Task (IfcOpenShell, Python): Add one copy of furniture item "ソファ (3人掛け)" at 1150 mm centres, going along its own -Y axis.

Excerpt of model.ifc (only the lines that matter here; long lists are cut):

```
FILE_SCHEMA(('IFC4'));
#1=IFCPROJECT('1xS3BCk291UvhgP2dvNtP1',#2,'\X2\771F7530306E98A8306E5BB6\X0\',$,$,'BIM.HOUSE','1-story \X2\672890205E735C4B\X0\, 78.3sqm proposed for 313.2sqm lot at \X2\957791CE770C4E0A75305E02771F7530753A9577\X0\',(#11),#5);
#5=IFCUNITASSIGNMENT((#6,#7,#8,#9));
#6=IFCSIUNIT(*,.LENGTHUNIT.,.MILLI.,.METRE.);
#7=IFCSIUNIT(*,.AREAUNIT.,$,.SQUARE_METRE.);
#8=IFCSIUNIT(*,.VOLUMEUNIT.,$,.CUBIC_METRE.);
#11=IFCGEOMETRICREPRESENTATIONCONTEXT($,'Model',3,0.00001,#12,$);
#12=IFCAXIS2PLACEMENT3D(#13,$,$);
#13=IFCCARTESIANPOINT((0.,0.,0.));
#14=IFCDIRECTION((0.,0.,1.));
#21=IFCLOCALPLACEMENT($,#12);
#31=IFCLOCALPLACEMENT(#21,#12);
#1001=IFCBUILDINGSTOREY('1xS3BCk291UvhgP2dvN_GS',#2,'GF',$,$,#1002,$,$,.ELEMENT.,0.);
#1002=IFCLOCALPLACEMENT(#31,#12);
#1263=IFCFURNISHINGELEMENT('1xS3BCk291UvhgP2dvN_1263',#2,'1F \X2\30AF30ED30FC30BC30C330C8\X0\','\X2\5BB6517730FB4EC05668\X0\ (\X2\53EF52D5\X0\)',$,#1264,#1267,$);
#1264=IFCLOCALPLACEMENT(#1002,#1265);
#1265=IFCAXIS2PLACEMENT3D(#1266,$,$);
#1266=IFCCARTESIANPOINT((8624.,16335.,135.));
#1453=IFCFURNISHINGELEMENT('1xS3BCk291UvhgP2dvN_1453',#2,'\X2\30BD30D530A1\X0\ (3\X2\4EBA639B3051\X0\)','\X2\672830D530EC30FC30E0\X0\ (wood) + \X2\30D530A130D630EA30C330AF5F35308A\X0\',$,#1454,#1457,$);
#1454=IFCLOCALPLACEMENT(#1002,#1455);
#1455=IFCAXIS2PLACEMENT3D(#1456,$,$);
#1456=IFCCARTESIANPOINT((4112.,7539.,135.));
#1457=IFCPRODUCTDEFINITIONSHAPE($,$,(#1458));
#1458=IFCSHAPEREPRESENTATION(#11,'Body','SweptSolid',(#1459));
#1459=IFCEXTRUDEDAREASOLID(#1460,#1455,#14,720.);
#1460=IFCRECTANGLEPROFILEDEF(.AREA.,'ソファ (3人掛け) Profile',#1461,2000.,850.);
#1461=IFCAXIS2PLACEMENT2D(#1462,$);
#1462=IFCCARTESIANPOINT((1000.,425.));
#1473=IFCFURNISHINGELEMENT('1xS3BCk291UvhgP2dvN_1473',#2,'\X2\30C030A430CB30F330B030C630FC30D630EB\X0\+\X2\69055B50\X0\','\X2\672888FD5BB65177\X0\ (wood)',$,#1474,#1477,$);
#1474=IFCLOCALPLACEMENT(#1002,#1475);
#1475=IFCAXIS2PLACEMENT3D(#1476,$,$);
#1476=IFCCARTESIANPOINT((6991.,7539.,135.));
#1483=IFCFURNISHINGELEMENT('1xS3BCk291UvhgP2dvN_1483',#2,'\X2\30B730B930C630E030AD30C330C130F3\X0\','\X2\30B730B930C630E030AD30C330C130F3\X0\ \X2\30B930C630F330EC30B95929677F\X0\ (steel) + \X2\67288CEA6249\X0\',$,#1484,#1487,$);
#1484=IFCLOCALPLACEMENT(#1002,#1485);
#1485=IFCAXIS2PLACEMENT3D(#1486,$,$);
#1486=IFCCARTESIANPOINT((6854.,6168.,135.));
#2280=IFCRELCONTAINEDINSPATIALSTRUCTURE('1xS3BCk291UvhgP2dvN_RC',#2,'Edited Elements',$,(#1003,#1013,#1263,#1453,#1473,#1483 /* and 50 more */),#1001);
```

```python
import ifcopenshell
import ifcopenshell.api.geometry
import ifcopenshell.api.root
import ifcopenshell.util.element
import ifcopenshell.util.placement
import ifcopenshell.util.unit

model = ifcopenshell.open("model.ifc")
unit_scale = ifcopenshell.util.unit.calculate_unit_scale(model)


def reuse_history(source, copy):
    """copy_class also copies each property set's owner history, people and application; keep the originals."""
    for rel in copy.IsDefinedBy:
        if rel.is_a("IfcRelDefinesByProperties") and (history := rel.RelatingPropertyDefinition.OwnerHistory):
            rel.RelatingPropertyDefinition.OwnerHistory = source.OwnerHistory
            ifcopenshell.util.element.remove_deep2(model, history)


source = model.by_id(1453)
base = ifcopenshell.util.placement.get_local_placement(source.ObjectPlacement)
step = -base[:3, 1] * 1.15 / unit_scale

for i in range(1, 2):
    copy = ifcopenshell.api.root.copy_class(model, product=source)
    copy.Representation = ifcopenshell.util.element.copy_deep(
        model, source.Representation, exclude=["IfcGeometricRepresentationContext", "IfcRepresentationMap"]
    )
    reuse_history(source, copy)
    matrix = base.copy()
    matrix[:3, 3] += i * step
    print("added at", matrix[:3, 3].round(3) + 0.0)
    ifcopenshell.api.geometry.edit_object_placement(model, product=copy, matrix=matrix, is_si=False)

model.write("model-out.ifc")
```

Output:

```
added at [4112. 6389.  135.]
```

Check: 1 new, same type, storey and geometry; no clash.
